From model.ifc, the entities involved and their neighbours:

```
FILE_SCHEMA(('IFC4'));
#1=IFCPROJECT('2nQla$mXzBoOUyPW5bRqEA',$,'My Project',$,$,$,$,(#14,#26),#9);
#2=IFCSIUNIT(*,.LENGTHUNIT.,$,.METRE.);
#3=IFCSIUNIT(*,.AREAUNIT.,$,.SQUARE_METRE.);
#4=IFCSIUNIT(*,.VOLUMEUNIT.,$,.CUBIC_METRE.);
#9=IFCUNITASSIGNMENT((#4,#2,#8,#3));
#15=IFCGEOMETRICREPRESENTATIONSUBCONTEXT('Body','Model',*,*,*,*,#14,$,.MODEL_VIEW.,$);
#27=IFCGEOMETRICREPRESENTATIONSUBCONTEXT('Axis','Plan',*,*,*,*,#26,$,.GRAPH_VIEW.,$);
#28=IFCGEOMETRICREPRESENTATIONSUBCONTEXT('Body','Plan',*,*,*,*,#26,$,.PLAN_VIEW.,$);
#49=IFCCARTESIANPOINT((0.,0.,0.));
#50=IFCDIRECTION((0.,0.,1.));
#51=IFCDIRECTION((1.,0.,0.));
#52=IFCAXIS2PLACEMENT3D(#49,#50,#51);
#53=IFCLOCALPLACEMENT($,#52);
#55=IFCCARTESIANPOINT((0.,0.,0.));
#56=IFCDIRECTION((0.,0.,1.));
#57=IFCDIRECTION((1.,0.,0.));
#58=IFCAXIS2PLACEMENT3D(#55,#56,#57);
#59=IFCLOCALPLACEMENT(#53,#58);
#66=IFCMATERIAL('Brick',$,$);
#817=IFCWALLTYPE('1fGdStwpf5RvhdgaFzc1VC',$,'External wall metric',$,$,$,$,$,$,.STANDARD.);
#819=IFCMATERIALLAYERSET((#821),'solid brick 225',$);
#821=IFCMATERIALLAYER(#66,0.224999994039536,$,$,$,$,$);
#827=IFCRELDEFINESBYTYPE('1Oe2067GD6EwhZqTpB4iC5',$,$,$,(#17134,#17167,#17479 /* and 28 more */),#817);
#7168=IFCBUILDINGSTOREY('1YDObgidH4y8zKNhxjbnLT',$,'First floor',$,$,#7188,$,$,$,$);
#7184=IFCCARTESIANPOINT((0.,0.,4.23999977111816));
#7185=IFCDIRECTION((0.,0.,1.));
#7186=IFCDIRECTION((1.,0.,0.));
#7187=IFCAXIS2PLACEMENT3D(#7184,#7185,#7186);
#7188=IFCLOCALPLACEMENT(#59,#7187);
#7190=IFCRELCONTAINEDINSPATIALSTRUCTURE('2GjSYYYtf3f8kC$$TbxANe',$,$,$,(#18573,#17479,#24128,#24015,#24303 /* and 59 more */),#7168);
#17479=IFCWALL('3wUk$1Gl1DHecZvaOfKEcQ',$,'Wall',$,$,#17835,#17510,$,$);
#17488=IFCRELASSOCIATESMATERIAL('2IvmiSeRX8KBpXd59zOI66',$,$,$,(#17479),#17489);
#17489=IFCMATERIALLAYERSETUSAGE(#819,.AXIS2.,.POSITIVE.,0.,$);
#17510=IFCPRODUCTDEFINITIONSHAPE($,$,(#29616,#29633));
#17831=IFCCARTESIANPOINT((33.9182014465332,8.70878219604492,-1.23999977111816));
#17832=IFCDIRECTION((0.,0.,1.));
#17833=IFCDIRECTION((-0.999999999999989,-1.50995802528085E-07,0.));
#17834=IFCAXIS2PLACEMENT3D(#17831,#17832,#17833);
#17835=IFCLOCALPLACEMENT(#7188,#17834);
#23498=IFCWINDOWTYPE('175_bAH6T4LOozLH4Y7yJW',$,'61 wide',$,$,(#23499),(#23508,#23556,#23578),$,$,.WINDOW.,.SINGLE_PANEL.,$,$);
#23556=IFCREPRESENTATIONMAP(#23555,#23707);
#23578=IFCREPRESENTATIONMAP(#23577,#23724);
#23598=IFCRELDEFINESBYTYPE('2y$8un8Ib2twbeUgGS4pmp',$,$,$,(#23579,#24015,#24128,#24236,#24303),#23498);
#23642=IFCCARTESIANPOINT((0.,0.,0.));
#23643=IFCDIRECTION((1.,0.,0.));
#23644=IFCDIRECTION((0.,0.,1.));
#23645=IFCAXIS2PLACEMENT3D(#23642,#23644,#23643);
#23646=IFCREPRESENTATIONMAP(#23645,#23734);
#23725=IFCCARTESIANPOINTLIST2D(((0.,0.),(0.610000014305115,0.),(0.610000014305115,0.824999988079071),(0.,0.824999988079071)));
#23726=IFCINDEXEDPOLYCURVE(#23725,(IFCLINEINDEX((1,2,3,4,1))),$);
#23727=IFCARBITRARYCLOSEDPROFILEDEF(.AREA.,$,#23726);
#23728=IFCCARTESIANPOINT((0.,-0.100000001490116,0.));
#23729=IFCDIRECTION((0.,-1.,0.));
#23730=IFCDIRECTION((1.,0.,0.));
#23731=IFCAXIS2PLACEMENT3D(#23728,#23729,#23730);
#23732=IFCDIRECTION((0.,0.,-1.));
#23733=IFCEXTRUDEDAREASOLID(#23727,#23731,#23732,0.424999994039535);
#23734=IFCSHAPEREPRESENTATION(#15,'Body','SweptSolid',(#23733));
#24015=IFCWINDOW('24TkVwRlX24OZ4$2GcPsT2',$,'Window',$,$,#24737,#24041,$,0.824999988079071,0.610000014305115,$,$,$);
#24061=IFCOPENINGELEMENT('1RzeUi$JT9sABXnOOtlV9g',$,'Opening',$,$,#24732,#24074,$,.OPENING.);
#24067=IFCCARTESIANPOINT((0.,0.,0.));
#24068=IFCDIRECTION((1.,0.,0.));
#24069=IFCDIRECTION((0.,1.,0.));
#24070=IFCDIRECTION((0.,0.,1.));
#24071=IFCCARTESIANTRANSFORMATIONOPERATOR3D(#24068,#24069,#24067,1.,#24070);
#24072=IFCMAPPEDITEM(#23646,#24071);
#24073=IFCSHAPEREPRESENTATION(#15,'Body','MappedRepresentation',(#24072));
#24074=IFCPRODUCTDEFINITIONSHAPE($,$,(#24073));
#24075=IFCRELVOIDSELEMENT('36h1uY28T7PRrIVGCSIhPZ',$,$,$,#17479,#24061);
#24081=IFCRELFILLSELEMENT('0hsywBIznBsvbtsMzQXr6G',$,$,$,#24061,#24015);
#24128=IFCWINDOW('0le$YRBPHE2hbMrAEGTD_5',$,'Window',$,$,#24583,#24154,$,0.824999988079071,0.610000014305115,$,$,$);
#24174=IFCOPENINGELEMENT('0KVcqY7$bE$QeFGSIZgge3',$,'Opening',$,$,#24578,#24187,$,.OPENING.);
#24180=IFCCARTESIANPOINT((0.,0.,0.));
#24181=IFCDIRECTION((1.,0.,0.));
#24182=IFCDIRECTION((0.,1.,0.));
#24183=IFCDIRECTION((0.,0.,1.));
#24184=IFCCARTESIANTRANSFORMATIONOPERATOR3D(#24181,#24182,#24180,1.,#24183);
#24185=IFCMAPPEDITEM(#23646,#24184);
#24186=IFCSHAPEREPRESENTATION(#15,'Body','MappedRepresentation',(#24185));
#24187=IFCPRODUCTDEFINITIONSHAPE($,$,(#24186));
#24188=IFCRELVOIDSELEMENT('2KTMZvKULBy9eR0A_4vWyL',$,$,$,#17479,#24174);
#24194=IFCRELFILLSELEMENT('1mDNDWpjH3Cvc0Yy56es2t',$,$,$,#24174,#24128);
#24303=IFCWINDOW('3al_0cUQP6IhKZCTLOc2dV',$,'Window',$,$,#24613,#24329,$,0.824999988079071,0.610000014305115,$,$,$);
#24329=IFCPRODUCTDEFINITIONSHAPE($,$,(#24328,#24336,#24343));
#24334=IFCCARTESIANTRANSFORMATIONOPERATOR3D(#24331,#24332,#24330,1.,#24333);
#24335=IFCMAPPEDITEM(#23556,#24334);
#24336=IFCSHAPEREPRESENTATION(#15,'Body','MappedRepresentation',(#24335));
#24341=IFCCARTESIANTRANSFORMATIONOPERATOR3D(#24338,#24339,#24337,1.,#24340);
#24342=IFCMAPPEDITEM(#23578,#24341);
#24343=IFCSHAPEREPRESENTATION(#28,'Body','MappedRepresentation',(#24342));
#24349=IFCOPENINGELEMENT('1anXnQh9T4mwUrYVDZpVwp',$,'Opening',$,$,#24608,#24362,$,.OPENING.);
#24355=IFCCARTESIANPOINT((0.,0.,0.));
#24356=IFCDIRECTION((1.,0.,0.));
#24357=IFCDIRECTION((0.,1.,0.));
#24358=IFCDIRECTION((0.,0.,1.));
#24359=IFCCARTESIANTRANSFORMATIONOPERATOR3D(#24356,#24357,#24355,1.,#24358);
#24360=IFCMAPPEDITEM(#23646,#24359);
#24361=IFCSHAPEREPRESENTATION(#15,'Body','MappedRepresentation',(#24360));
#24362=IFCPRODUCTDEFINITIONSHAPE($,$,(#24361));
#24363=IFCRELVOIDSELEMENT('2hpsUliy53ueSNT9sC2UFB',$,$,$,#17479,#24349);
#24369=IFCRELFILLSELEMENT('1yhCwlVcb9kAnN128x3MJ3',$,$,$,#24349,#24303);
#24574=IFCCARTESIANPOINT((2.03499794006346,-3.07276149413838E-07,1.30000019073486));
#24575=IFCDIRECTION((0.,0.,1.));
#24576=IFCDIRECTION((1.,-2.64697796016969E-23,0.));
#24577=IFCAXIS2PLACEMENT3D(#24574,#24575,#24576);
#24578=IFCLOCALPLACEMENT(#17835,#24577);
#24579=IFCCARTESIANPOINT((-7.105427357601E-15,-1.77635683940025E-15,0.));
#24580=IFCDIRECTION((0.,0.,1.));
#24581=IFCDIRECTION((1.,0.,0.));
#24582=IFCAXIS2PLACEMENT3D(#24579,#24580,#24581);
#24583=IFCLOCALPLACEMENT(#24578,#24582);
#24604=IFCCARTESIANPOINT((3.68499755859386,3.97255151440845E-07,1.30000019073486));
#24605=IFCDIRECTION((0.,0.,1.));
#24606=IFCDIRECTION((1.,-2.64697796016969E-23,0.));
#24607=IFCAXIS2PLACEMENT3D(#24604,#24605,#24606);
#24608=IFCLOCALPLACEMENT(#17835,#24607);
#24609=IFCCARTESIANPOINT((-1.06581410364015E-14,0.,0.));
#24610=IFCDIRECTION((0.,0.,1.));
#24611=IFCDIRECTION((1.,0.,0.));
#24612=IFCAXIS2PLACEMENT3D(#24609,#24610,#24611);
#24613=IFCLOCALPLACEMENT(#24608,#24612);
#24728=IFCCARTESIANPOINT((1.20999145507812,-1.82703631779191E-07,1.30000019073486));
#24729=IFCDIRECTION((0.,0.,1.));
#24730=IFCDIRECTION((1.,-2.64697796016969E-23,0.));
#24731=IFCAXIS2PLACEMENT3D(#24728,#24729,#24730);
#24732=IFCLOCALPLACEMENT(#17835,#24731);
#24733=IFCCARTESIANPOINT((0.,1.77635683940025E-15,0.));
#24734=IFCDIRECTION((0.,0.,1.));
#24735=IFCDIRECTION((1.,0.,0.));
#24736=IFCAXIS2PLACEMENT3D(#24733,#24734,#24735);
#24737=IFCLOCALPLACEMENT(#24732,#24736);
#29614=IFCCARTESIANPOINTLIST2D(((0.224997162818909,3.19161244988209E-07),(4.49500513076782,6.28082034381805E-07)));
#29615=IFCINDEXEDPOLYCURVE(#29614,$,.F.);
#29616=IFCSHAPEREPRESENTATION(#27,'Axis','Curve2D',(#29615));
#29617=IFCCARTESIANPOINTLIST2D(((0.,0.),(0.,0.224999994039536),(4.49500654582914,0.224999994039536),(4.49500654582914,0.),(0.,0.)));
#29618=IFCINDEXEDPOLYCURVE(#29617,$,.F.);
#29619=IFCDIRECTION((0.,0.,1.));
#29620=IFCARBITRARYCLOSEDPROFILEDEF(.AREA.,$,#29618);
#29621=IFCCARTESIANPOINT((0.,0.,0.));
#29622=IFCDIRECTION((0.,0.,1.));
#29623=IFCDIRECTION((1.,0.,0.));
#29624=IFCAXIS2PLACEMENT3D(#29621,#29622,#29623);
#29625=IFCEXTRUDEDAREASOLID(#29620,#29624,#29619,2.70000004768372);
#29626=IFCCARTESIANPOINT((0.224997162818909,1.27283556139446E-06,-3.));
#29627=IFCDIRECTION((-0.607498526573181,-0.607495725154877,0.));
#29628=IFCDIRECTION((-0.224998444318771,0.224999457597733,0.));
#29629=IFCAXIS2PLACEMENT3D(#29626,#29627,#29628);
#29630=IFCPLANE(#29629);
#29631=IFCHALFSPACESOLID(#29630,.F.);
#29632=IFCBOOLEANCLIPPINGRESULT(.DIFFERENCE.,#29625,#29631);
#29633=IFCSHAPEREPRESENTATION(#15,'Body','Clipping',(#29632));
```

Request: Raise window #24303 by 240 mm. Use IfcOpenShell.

```python
import numpy as np
import ifcopenshell
import ifcopenshell.api.geometry
import ifcopenshell.util.placement
import ifcopenshell.util.unit

model = ifcopenshell.open("model.ifc")
unit_scale = ifcopenshell.util.unit.calculate_unit_scale(model)

window = model.by_guid("3al_0cUQP6IhKZCTLOc2dV")
opening = window.FillsVoids[0].RelatingOpeningElement
dz = 0.24 / unit_scale

shift = np.array([0.0, 0.0, dz])
# The window is placed relative to its opening, so it follows when the opening moves.
matrix = ifcopenshell.util.placement.get_local_placement(opening.ObjectPlacement)
matrix[:3, 3] += shift
ifcopenshell.api.geometry.edit_object_placement(
    model, product=opening, matrix=matrix, is_si=False, should_transform_children=True
)

print(f"moved by {dz * unit_scale:+.3f} m")

model.write("model-out.ifc")
```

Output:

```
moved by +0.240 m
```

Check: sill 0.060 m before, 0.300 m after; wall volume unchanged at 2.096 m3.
